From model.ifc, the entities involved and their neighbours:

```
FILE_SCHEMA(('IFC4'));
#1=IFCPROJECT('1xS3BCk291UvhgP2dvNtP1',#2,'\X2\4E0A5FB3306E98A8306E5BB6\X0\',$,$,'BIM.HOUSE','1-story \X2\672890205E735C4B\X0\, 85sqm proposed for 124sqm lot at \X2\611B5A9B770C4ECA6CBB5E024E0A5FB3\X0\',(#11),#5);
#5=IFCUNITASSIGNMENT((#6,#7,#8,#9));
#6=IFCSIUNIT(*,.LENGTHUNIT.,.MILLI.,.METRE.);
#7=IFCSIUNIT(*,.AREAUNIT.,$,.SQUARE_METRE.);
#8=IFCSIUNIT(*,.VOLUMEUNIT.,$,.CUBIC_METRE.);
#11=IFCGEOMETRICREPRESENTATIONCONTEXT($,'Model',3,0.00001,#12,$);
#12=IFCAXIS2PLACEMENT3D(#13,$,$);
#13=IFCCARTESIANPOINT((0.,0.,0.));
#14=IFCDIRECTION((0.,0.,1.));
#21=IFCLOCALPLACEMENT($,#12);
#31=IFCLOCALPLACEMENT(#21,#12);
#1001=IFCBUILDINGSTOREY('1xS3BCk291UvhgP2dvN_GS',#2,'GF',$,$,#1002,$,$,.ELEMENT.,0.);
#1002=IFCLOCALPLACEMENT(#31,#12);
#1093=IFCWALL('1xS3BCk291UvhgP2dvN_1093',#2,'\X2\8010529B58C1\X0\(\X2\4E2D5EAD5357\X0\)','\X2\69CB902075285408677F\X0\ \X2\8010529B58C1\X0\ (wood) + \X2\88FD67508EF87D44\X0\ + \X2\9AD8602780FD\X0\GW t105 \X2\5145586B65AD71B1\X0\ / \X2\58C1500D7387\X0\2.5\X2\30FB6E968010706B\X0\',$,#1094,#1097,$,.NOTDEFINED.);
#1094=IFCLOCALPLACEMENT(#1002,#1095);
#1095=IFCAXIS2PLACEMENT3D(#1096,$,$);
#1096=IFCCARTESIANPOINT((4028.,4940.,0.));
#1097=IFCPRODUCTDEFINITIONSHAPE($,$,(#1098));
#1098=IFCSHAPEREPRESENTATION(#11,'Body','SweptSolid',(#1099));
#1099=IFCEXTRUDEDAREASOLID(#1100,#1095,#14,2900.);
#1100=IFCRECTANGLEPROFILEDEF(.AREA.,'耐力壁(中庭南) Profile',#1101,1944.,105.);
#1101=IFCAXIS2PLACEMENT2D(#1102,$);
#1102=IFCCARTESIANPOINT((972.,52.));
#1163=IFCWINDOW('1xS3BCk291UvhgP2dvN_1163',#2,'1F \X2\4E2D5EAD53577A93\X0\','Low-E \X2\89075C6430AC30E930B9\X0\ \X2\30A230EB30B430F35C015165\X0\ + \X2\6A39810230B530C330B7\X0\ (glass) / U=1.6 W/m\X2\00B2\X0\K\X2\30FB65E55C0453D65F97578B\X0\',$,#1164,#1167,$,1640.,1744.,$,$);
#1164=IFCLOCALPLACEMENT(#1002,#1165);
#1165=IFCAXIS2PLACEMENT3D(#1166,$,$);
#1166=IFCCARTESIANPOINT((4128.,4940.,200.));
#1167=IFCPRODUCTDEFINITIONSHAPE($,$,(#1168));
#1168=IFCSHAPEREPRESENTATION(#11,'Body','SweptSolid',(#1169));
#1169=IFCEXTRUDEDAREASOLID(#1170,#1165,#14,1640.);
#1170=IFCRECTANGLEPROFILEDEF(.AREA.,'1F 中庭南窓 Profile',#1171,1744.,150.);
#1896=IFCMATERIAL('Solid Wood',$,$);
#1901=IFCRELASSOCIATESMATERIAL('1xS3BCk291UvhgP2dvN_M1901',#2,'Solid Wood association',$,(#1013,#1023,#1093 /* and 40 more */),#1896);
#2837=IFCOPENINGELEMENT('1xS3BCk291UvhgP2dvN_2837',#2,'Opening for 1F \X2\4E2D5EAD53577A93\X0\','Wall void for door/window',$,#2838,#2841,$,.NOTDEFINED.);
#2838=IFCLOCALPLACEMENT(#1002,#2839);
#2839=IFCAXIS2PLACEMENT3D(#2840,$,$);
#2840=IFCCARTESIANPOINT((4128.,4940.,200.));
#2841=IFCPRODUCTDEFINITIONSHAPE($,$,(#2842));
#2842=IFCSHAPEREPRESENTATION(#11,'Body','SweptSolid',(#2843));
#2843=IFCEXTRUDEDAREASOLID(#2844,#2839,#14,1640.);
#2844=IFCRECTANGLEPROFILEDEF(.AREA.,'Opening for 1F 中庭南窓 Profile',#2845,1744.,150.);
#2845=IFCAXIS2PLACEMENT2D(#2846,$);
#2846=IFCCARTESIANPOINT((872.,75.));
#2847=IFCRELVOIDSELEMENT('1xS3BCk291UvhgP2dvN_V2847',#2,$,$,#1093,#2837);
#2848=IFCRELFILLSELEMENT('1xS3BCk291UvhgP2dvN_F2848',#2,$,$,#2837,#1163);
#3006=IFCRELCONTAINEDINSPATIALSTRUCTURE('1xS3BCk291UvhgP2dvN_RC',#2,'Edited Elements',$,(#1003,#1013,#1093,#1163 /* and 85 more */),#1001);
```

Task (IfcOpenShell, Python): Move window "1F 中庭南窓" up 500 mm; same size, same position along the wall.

```python
import numpy as np
import ifcopenshell
import ifcopenshell.api.geometry
import ifcopenshell.util.placement
import ifcopenshell.util.unit

model = ifcopenshell.open("model.ifc")
unit_scale = ifcopenshell.util.unit.calculate_unit_scale(model)

window = model.by_guid("1xS3BCk291UvhgP2dvN_1163")
opening = window.FillsVoids[0].RelatingOpeningElement
dz = 500.0

shift = np.array([0.0, 0.0, dz])
# The window is not placed relative to its opening, so move both.
for product in (opening, window):
    matrix = ifcopenshell.util.placement.get_local_placement(product.ObjectPlacement)
    matrix[:3, 3] += shift
    ifcopenshell.api.geometry.edit_object_placement(model, product=product, matrix=matrix, is_si=False)

print(f"moved by {dz * unit_scale:+.3f} m")

model.write("model_edited.ifc")
```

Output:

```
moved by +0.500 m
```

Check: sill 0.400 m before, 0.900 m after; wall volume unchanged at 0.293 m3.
